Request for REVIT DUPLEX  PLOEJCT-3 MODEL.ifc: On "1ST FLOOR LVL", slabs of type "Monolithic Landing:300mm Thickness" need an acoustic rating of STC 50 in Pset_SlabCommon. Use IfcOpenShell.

First a look at what the model holds.

```python
import ifcopenshell
import ifcopenshell.util.element

model = ifcopenshell.open("REVIT DUPLEX  PLOEJCT-3 MODEL.ifc")
print(model.schema)
storey = next(s for s in model.by_type("IfcBuildingStorey") if s.Name == "1ST FLOOR LVL")
slabs = [e for e in ifcopenshell.util.element.get_decomposition(storey) if e.is_a("IfcSlab")]
seen = {}
for e in slabs:
    element_type = ifcopenshell.util.element.get_type(e)
    key = (element_type.Name if element_type != e and element_type else None, ifcopenshell.util.element.get_pset(e, "Pset_SlabCommon", "AcousticRating"))
    seen[key] = seen.get(key, 0) + 1
for (name, value), count in sorted(seen.items(), key=str):
    print(count, "x", name, "|", value)
```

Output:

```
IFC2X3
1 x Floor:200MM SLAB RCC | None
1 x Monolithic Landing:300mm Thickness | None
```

```python
import ifcopenshell
import ifcopenshell.api.pset
import ifcopenshell.util.element

model = ifcopenshell.open("REVIT DUPLEX  PLOEJCT-3 MODEL.ifc")

storey = next(s for s in model.by_type("IfcBuildingStorey") if s.Name == "1ST FLOOR LVL")
slabs = [e for e in ifcopenshell.util.element.get_decomposition(storey) if e.is_a("IfcSlab")]

count = 0
for e in slabs:
    element_type = ifcopenshell.util.element.get_type(e)
    if element_type in (None, e) or element_type.Name != "Monolithic Landing:300mm Thickness":
        continue
    # add_pset returns the element's existing set when there is one.
    pset = ifcopenshell.api.pset.add_pset(model, product=e, name="Pset_SlabCommon")
    ifcopenshell.api.pset.edit_pset(model, pset=pset, properties={"AcousticRating": "STC 50"})
    count += 1

print(count, "slabs updated")

model.write("REVIT DUPLEX  PLOEJCT-3 MODEL_v2.ifc")
```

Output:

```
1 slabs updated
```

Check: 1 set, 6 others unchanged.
